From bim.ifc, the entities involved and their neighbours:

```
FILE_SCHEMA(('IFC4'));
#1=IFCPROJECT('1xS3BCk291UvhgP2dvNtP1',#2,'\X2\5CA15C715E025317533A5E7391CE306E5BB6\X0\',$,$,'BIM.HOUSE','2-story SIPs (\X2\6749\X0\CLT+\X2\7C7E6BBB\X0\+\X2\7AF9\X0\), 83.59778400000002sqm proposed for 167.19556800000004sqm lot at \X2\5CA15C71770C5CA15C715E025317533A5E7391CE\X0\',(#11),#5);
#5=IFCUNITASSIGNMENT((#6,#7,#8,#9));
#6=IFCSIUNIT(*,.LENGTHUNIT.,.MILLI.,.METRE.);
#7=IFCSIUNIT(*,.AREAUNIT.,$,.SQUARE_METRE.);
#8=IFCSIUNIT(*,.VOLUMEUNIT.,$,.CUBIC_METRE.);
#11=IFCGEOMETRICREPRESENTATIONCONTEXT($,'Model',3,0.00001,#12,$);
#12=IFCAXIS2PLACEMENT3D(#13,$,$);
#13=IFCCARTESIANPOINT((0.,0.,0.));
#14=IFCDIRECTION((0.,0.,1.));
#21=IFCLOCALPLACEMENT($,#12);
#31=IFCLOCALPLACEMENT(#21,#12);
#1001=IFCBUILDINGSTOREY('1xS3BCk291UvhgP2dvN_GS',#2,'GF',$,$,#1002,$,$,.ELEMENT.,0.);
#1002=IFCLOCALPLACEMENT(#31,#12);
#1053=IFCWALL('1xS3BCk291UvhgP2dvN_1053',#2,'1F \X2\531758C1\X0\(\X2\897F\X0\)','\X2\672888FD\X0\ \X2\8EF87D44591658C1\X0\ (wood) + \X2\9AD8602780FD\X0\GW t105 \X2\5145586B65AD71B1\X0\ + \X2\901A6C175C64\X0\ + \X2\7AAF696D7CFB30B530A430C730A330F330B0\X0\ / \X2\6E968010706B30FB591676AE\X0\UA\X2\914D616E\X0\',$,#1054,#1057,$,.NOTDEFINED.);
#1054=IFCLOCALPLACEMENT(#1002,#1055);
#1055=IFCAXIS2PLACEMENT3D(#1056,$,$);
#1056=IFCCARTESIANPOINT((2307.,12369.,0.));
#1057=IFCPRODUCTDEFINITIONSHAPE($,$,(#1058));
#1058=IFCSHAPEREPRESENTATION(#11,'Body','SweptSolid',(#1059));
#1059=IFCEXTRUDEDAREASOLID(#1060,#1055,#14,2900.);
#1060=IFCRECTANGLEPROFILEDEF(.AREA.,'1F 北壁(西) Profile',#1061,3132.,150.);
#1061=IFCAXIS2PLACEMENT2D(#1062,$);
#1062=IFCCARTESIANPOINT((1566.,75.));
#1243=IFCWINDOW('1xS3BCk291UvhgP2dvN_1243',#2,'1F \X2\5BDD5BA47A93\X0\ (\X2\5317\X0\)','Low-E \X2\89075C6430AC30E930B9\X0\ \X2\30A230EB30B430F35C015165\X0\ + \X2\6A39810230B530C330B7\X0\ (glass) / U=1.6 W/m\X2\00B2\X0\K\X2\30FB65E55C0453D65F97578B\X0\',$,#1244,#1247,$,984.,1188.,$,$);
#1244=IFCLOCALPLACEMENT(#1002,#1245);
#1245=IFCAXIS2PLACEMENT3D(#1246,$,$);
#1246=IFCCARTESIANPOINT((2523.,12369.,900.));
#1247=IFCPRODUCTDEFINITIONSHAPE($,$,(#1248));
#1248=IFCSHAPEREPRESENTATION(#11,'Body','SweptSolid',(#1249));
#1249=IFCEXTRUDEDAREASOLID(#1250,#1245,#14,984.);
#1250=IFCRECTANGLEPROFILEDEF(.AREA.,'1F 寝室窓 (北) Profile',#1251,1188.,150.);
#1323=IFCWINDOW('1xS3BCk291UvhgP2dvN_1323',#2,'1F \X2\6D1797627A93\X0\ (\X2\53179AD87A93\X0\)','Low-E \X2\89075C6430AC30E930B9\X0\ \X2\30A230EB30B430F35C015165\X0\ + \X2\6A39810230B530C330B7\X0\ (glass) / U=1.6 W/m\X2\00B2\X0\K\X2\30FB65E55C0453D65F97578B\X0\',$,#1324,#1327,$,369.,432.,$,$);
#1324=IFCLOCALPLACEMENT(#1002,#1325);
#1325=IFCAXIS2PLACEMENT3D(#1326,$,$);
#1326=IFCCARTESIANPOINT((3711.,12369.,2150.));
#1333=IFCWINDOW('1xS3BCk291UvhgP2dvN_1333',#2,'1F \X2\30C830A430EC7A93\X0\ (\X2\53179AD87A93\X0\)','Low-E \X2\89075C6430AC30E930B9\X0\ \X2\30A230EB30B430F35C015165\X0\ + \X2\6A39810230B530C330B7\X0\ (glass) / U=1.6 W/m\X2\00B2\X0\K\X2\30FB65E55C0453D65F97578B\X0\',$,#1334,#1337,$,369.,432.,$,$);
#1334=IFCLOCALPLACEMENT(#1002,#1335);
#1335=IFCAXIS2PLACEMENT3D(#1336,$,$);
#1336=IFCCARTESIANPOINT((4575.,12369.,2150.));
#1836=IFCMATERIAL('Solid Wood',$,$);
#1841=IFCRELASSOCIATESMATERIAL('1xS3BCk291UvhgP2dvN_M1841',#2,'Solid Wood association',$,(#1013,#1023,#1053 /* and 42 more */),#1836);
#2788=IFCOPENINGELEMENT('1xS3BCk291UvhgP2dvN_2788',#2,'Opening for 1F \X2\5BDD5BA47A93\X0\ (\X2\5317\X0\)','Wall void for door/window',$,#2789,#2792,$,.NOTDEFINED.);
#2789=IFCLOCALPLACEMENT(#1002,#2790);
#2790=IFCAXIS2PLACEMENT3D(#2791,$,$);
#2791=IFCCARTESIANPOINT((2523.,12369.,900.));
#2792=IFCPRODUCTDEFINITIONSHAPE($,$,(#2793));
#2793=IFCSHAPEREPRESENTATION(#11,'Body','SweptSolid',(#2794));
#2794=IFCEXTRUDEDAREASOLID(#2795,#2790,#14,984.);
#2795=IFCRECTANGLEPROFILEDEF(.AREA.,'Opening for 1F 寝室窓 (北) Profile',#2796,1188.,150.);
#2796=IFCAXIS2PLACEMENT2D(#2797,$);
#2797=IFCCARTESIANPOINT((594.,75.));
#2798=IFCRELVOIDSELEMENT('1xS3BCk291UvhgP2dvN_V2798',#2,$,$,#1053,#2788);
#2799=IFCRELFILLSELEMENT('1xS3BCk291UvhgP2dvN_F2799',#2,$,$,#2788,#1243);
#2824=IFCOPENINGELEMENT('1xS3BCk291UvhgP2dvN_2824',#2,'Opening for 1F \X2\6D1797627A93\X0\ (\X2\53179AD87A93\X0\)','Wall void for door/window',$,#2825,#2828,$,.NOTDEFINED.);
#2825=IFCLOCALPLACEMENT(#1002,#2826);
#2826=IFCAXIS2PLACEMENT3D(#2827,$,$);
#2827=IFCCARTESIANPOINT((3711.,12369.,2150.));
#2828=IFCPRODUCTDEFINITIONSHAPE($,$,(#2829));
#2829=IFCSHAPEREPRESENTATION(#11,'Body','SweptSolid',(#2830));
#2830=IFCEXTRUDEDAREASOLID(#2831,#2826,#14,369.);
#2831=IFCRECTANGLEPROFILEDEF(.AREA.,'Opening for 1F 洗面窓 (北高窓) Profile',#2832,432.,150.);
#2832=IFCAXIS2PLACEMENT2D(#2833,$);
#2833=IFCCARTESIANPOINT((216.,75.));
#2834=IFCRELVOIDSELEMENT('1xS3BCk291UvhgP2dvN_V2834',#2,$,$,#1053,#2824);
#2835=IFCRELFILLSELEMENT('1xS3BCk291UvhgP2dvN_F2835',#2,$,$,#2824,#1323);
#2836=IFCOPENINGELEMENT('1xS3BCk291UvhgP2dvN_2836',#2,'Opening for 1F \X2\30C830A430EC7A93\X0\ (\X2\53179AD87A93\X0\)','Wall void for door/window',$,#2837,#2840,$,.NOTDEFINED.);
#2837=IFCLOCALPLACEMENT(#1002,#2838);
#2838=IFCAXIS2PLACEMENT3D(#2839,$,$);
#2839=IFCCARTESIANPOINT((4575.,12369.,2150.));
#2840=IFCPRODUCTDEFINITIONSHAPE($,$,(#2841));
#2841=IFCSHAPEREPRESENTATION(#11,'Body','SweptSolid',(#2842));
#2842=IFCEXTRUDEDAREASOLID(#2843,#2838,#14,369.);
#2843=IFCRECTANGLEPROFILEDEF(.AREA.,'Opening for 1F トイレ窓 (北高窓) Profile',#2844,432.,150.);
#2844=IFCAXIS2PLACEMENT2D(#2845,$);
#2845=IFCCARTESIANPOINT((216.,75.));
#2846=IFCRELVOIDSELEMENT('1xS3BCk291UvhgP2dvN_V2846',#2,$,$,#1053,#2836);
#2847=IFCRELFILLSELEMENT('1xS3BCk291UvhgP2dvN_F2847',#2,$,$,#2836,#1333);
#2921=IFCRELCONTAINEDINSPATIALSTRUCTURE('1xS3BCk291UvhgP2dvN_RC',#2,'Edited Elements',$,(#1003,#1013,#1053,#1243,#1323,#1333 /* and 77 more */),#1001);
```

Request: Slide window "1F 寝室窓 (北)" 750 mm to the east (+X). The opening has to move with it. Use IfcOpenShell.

```python
import ifcopenshell
import ifcopenshell.api.geometry
import ifcopenshell.util.placement
import ifcopenshell.util.unit

model = ifcopenshell.open("bim.ifc")
unit_scale = ifcopenshell.util.unit.calculate_unit_scale(model)

window = model.by_guid("1xS3BCk291UvhgP2dvN_1243")
opening = window.FillsVoids[0].RelatingOpeningElement
wall = opening.VoidsElements[0].RelatingBuildingElement

wall_matrix = ifcopenshell.util.placement.get_local_placement(wall.ObjectPlacement)
shift = wall_matrix[:3, 0] * 0.75 / unit_scale
before = ifcopenshell.util.placement.get_local_placement(window.ObjectPlacement)[:3, 3].copy()

# The window is not placed relative to its opening, so move both.
for product in (opening, window):
    matrix = ifcopenshell.util.placement.get_local_placement(product.ObjectPlacement)
    matrix[:3, 3] += shift
    ifcopenshell.api.geometry.edit_object_placement(model, product=product, matrix=matrix, is_si=False)

after = ifcopenshell.util.placement.get_local_placement(window.ObjectPlacement)[:3, 3]
print("window moved by", (after - before).round(3) + 0.0)

model.write("bim_updated.ifc")
```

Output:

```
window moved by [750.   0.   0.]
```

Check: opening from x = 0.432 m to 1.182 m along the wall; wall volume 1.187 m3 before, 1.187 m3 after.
